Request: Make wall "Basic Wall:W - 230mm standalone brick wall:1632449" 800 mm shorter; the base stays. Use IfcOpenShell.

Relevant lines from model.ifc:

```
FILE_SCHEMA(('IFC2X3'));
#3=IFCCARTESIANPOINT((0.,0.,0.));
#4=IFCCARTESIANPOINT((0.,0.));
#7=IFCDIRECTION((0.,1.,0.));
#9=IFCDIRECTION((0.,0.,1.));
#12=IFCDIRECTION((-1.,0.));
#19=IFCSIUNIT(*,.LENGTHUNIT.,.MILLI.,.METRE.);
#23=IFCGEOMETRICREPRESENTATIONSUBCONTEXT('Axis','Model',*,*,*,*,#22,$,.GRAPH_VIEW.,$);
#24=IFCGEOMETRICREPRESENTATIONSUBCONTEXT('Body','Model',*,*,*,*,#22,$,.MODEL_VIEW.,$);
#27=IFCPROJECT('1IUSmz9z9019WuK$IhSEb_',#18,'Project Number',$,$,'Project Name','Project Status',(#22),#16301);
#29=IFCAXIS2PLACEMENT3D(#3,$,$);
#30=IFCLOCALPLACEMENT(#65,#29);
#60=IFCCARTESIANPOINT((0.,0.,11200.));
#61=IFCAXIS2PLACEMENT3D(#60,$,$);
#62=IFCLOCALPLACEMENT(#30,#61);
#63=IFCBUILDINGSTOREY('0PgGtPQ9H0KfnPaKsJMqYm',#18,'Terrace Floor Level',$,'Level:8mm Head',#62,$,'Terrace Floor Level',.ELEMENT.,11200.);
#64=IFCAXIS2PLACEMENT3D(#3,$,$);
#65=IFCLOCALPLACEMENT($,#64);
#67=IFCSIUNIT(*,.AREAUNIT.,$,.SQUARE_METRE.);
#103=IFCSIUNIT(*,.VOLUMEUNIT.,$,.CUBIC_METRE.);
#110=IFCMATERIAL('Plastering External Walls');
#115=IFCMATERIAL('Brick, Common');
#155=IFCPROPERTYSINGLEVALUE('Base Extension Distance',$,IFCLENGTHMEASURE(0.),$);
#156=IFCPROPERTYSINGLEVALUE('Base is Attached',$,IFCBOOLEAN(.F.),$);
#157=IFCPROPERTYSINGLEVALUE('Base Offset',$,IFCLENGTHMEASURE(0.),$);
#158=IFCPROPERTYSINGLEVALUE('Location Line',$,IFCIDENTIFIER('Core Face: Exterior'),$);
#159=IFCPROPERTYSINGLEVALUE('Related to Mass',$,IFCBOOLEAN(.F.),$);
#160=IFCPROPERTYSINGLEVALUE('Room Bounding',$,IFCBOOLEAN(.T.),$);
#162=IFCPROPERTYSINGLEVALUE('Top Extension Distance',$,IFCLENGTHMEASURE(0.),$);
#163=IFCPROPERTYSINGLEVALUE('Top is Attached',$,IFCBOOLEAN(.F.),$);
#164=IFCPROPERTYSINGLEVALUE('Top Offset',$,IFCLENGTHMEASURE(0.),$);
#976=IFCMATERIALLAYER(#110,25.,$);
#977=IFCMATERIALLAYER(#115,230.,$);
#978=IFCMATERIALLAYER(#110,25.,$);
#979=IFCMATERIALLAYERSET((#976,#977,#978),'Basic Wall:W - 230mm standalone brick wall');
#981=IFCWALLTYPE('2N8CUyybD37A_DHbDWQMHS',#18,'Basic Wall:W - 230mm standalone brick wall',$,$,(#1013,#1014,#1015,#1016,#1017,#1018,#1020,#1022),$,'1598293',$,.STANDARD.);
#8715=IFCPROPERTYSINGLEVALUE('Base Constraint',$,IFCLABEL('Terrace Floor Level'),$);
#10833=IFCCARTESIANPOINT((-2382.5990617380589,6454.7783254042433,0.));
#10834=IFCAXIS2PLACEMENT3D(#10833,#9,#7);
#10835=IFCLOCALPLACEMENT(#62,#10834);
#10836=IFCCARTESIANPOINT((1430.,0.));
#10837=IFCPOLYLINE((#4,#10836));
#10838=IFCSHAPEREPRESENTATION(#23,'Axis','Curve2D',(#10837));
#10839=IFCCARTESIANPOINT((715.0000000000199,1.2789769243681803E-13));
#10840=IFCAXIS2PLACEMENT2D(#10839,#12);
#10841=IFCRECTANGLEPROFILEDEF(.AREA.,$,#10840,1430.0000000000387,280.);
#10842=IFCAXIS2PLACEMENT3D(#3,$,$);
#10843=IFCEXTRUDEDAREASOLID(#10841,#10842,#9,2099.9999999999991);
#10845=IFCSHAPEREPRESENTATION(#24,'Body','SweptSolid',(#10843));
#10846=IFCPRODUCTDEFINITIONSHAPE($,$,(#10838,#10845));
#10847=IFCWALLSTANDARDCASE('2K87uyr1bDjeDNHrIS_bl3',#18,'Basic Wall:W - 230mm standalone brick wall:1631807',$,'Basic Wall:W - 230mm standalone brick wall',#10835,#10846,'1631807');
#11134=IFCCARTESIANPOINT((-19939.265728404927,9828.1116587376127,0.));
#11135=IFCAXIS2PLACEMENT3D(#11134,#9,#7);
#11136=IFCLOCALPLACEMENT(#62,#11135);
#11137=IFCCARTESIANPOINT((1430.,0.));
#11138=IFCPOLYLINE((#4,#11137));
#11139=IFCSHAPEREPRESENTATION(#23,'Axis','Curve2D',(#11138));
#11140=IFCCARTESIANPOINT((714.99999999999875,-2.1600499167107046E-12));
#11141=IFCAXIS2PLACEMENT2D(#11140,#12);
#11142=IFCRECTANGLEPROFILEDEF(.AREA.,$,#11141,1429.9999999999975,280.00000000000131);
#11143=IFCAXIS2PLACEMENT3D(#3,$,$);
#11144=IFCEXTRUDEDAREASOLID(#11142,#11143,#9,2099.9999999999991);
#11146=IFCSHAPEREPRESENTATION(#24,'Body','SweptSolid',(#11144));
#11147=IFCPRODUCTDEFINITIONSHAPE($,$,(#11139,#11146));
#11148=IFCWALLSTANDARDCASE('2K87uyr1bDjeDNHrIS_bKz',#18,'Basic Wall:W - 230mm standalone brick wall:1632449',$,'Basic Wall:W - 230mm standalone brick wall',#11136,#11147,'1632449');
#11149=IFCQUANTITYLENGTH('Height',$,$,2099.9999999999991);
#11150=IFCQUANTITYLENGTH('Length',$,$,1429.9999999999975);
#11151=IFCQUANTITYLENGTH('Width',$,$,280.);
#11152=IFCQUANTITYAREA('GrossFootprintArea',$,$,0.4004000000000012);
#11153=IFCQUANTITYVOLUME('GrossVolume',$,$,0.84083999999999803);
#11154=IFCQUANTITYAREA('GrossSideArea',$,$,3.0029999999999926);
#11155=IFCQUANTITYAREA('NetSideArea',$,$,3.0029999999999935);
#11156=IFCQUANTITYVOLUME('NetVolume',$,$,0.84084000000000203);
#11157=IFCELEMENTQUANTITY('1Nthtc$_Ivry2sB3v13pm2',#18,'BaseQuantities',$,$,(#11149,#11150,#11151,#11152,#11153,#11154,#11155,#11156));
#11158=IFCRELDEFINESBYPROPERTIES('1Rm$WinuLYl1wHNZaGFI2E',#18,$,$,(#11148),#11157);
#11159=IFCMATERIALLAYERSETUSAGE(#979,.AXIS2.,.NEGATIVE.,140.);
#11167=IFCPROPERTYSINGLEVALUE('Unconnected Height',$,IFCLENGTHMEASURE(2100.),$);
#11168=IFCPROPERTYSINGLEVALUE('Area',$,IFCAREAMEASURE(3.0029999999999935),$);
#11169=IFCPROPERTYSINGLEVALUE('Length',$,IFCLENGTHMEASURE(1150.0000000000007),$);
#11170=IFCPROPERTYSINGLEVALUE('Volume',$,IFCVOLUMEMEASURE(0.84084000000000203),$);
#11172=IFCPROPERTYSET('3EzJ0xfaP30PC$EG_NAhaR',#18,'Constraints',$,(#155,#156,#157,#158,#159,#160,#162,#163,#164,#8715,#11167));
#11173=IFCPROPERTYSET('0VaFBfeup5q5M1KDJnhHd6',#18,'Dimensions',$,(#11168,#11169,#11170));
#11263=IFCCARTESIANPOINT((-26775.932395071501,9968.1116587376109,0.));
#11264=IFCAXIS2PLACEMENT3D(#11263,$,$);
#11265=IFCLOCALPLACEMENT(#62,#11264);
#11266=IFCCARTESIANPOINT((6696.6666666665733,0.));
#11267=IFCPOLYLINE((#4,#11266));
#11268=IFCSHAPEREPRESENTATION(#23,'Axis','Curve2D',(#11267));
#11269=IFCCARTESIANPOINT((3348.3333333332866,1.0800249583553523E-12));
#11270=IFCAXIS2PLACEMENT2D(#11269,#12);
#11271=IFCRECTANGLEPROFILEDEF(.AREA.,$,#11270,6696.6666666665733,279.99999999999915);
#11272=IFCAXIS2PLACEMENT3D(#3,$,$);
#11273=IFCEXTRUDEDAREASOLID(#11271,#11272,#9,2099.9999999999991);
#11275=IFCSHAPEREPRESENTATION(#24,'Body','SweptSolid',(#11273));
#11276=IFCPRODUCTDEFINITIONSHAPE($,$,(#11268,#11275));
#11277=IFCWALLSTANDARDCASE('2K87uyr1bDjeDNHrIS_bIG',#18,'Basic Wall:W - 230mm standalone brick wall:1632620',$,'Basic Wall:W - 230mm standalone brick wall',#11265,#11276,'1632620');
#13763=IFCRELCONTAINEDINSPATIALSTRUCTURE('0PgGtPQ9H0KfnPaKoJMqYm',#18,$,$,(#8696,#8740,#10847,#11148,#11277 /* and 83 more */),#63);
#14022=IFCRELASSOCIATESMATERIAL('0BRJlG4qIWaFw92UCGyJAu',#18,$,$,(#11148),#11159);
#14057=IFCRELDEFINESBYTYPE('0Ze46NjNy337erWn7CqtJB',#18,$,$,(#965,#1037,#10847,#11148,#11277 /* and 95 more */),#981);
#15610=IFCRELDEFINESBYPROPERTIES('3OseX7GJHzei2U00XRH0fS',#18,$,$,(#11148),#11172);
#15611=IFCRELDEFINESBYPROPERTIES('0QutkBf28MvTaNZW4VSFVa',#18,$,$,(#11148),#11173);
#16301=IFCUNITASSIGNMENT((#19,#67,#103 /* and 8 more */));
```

```python
import ifcopenshell
import ifcopenshell.api.pset
import ifcopenshell.geom
import ifcopenshell.util.element
import ifcopenshell.util.representation
import ifcopenshell.util.shape
import ifcopenshell.util.unit

model = ifcopenshell.open("model.ifc")
unit_scale = ifcopenshell.util.unit.calculate_unit_scale(model)
area_scale = ifcopenshell.util.unit.calculate_unit_scale(model, "AREAUNIT")
volume_scale = ifcopenshell.util.unit.calculate_unit_scale(model, "VOLUMEUNIT")
settings = ifcopenshell.geom.settings()


def volume(element):
    """Net volume in cubic metres, openings subtracted."""
    shape = ifcopenshell.geom.create_shape(settings, element)
    return ifcopenshell.util.shape.get_volume(shape.geometry)


wall = model.by_guid("2K87uyr1bDjeDNHrIS_bKz")
before = volume(wall)

body = ifcopenshell.util.representation.get_representation(wall, "Model", "Body")
solid = body.Items[0]
old_height = solid.Depth
solid.Depth -= 800.0
after = volume(wall)
thickness = 0.28  # wall thickness in metres

# Update the stored height, areas and volumes.
qto = model.by_id(ifcopenshell.util.element.get_pset(wall, "BaseQuantities", should_inherit=False)["id"])
ifcopenshell.api.pset.edit_qto(model, qto=qto, properties={
    "Height": solid.Depth,
    "GrossVolume": ifcopenshell.util.element.get_pset(wall, "BaseQuantities", "GrossVolume") * solid.Depth / old_height,
    "GrossSideArea": ifcopenshell.util.element.get_pset(wall, "BaseQuantities", "GrossSideArea") * solid.Depth / old_height,
    "NetSideArea": after / thickness / area_scale,
    "NetVolume": after / volume_scale,
})
pset = model.by_id(ifcopenshell.util.element.get_pset(wall, "Constraints", should_inherit=False)["id"])
ifcopenshell.api.pset.edit_pset(model, pset=pset, properties={
    "Unconnected Height": model.create_entity("IfcLengthMeasure", solid.Depth),
})
pset = model.by_id(ifcopenshell.util.element.get_pset(wall, "Dimensions", should_inherit=False)["id"])
ifcopenshell.api.pset.edit_pset(model, pset=pset, properties={
    "Area": model.create_entity("IfcAreaMeasure", after / thickness / area_scale),
    "Volume": model.create_entity("IfcVolumeMeasure", after / volume_scale),
})

print(f"height {old_height:g} -> {solid.Depth:g}, volume {before:.3f} -> {after:.3f} m3")

model.write("model_updated.ifc")
```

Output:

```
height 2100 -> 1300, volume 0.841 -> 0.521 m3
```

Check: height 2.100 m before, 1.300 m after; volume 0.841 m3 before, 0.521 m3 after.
